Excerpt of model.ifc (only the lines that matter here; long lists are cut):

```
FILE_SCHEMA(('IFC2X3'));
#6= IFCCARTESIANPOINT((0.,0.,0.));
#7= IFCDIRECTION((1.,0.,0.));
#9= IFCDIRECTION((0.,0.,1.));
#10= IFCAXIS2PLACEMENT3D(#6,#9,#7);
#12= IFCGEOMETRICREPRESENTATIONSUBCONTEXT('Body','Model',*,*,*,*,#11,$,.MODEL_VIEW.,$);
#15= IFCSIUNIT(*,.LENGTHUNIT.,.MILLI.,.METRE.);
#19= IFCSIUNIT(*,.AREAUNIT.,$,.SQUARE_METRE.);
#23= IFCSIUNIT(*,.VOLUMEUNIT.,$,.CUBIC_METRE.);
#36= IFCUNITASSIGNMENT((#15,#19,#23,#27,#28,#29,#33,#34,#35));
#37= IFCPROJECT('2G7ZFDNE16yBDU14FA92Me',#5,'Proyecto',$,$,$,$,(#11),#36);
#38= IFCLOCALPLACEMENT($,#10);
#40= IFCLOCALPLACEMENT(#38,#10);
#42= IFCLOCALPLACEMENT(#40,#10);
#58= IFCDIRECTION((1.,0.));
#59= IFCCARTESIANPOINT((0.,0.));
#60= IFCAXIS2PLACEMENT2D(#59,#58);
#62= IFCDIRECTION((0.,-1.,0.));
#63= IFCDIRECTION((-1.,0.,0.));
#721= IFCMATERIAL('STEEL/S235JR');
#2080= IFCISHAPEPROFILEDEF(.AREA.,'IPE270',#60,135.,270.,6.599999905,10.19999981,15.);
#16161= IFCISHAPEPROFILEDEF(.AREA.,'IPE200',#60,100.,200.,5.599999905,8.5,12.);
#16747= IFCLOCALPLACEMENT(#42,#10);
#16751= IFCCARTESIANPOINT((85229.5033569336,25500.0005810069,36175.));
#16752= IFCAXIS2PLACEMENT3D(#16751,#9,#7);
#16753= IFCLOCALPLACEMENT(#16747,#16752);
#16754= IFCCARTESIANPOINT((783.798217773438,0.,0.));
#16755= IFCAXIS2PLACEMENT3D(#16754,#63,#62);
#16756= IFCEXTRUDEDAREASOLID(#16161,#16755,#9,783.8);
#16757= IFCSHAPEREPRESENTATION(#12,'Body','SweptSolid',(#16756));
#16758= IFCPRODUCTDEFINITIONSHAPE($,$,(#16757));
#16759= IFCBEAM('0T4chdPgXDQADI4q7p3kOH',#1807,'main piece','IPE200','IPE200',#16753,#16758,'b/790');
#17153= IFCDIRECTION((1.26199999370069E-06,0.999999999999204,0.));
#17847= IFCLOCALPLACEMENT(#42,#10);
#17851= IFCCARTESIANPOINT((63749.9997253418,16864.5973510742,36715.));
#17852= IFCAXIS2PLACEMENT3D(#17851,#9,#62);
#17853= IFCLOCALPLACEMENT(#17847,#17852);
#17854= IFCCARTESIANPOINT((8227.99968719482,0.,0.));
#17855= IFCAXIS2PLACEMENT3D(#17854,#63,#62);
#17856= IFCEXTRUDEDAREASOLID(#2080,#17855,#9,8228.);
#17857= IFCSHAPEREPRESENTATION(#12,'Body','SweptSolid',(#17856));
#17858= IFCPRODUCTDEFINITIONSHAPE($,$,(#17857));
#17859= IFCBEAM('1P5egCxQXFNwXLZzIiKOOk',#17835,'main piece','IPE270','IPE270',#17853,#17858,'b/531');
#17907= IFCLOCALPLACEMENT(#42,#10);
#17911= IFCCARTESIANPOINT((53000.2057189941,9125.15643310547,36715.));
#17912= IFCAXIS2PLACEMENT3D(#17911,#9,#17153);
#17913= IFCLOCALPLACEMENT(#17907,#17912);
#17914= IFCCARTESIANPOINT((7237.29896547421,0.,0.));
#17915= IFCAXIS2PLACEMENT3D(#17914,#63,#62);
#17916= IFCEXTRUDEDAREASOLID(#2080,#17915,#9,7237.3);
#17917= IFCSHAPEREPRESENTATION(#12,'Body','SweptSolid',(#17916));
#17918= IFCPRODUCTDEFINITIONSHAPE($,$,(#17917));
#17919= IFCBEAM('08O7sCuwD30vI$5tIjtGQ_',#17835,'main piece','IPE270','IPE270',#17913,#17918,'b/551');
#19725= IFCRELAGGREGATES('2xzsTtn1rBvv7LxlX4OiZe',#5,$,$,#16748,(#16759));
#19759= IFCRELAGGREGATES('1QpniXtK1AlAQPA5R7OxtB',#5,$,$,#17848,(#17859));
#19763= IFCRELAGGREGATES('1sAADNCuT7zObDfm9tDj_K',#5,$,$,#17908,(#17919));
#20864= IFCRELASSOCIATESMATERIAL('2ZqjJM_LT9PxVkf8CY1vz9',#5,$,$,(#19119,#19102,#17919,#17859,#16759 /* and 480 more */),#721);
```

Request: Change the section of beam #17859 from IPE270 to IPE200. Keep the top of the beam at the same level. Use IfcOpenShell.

```python
import ifcopenshell
import ifcopenshell.util.element
import ifcopenshell.util.representation

model = ifcopenshell.open("model.ifc")

member = model.by_guid("1P5egCxQXFNwXLZzIiKOOk")
source = next(p for p in model.by_type("IfcIShapeProfileDef") if p.ProfileName == "IPE200")

body = ifcopenshell.util.representation.get_representation(member, "Model", "Body")
solid = body.Items[0]
old_profile = solid.SweptArea

# Copy the section's sizes but keep this member's own profile position.
profile = ifcopenshell.util.element.copy(model, source)
# Profiles are centred, so shift by half the change in depth to hold the top.
shift = (old_profile.OverallDepth - profile.OverallDepth) / 2
x, y = old_profile.Position.Location.Coordinates
up = (0.0, 1.0)  # upwards, in the solid's own plane
location = model.createIfcCartesianPoint((x + up[0] * shift, y + up[1] * shift))
profile.Position = model.createIfcAxis2Placement2D(location, old_profile.Position.RefDirection)
solid.SweptArea = profile
if not model.get_total_inverses(old_profile):
    ifcopenshell.util.element.remove_deep2(model, old_profile)
member.Description = member.Description.replace("IPE270", "IPE200")
member.ObjectType = member.ObjectType.replace("IPE270", "IPE200")

print(solid.SweptArea)

model.write("model_updated.ifc")
```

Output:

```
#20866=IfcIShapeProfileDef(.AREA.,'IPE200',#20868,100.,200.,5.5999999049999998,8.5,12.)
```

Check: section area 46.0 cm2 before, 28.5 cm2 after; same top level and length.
